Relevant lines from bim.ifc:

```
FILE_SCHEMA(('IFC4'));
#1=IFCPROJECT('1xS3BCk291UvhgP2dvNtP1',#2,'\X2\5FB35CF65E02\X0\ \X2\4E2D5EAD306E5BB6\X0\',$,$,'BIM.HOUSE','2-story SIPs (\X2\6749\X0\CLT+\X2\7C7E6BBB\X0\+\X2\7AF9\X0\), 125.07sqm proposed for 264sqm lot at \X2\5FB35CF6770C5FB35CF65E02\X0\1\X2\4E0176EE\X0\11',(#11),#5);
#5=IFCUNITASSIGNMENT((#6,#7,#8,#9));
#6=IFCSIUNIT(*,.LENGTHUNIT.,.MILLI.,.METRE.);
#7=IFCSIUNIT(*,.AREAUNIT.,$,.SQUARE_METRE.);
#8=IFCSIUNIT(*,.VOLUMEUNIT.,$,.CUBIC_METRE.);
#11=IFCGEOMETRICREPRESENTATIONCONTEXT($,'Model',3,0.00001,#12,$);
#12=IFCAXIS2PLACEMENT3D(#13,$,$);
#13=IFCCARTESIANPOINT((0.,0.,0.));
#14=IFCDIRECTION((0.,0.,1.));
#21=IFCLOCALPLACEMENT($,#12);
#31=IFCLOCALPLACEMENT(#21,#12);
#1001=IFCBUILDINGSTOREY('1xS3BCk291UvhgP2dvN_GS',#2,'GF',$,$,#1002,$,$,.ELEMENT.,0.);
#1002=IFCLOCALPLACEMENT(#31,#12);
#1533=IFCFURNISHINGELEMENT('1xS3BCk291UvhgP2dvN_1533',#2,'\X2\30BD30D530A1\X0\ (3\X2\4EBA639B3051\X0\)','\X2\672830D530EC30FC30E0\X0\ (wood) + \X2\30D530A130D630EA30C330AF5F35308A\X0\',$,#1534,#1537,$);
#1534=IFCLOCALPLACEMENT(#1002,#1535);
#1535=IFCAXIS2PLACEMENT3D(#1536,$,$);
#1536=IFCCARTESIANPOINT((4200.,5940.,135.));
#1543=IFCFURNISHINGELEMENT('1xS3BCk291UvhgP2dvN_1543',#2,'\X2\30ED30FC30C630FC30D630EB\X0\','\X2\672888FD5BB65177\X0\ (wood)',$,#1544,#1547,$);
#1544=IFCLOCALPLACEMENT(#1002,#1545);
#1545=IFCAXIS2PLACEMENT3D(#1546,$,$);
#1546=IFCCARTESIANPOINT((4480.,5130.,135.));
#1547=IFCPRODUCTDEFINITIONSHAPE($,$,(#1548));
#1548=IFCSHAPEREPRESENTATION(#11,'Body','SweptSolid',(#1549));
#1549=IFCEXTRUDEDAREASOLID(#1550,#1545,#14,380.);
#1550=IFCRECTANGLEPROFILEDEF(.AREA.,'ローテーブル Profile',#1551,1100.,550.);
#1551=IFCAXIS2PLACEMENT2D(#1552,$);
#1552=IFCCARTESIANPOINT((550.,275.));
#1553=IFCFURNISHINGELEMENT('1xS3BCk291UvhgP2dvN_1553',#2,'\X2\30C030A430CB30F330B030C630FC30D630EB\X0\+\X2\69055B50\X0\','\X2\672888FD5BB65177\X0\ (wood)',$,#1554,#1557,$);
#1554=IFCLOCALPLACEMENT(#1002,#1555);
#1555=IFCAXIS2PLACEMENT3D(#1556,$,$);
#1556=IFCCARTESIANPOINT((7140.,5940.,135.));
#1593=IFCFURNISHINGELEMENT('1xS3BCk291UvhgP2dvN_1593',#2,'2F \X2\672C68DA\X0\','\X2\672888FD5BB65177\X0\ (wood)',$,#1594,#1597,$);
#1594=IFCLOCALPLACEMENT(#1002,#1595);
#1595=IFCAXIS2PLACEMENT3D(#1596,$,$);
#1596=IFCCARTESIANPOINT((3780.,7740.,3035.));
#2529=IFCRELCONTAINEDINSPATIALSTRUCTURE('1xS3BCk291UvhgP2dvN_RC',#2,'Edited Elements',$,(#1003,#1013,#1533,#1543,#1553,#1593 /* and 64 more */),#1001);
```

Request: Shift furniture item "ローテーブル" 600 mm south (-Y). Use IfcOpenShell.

```python
import ifcopenshell
import ifcopenshell.api.geometry
import ifcopenshell.util.placement

model = ifcopenshell.open("bim.ifc")

item = model.by_guid("1xS3BCk291UvhgP2dvN_1543")
matrix = ifcopenshell.util.placement.get_local_placement(item.ObjectPlacement)
matrix[1, 3] -= 600.0
ifcopenshell.api.geometry.edit_object_placement(model, product=item, matrix=matrix, is_si=False)

print(ifcopenshell.util.placement.get_local_placement(item.ObjectPlacement).round(3) + 0.0)

model.write("bim-out.ifc")
```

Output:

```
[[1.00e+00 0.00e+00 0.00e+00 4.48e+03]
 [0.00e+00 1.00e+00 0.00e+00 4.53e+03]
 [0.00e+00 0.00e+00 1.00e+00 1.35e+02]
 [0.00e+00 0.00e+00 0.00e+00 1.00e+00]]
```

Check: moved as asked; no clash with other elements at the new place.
